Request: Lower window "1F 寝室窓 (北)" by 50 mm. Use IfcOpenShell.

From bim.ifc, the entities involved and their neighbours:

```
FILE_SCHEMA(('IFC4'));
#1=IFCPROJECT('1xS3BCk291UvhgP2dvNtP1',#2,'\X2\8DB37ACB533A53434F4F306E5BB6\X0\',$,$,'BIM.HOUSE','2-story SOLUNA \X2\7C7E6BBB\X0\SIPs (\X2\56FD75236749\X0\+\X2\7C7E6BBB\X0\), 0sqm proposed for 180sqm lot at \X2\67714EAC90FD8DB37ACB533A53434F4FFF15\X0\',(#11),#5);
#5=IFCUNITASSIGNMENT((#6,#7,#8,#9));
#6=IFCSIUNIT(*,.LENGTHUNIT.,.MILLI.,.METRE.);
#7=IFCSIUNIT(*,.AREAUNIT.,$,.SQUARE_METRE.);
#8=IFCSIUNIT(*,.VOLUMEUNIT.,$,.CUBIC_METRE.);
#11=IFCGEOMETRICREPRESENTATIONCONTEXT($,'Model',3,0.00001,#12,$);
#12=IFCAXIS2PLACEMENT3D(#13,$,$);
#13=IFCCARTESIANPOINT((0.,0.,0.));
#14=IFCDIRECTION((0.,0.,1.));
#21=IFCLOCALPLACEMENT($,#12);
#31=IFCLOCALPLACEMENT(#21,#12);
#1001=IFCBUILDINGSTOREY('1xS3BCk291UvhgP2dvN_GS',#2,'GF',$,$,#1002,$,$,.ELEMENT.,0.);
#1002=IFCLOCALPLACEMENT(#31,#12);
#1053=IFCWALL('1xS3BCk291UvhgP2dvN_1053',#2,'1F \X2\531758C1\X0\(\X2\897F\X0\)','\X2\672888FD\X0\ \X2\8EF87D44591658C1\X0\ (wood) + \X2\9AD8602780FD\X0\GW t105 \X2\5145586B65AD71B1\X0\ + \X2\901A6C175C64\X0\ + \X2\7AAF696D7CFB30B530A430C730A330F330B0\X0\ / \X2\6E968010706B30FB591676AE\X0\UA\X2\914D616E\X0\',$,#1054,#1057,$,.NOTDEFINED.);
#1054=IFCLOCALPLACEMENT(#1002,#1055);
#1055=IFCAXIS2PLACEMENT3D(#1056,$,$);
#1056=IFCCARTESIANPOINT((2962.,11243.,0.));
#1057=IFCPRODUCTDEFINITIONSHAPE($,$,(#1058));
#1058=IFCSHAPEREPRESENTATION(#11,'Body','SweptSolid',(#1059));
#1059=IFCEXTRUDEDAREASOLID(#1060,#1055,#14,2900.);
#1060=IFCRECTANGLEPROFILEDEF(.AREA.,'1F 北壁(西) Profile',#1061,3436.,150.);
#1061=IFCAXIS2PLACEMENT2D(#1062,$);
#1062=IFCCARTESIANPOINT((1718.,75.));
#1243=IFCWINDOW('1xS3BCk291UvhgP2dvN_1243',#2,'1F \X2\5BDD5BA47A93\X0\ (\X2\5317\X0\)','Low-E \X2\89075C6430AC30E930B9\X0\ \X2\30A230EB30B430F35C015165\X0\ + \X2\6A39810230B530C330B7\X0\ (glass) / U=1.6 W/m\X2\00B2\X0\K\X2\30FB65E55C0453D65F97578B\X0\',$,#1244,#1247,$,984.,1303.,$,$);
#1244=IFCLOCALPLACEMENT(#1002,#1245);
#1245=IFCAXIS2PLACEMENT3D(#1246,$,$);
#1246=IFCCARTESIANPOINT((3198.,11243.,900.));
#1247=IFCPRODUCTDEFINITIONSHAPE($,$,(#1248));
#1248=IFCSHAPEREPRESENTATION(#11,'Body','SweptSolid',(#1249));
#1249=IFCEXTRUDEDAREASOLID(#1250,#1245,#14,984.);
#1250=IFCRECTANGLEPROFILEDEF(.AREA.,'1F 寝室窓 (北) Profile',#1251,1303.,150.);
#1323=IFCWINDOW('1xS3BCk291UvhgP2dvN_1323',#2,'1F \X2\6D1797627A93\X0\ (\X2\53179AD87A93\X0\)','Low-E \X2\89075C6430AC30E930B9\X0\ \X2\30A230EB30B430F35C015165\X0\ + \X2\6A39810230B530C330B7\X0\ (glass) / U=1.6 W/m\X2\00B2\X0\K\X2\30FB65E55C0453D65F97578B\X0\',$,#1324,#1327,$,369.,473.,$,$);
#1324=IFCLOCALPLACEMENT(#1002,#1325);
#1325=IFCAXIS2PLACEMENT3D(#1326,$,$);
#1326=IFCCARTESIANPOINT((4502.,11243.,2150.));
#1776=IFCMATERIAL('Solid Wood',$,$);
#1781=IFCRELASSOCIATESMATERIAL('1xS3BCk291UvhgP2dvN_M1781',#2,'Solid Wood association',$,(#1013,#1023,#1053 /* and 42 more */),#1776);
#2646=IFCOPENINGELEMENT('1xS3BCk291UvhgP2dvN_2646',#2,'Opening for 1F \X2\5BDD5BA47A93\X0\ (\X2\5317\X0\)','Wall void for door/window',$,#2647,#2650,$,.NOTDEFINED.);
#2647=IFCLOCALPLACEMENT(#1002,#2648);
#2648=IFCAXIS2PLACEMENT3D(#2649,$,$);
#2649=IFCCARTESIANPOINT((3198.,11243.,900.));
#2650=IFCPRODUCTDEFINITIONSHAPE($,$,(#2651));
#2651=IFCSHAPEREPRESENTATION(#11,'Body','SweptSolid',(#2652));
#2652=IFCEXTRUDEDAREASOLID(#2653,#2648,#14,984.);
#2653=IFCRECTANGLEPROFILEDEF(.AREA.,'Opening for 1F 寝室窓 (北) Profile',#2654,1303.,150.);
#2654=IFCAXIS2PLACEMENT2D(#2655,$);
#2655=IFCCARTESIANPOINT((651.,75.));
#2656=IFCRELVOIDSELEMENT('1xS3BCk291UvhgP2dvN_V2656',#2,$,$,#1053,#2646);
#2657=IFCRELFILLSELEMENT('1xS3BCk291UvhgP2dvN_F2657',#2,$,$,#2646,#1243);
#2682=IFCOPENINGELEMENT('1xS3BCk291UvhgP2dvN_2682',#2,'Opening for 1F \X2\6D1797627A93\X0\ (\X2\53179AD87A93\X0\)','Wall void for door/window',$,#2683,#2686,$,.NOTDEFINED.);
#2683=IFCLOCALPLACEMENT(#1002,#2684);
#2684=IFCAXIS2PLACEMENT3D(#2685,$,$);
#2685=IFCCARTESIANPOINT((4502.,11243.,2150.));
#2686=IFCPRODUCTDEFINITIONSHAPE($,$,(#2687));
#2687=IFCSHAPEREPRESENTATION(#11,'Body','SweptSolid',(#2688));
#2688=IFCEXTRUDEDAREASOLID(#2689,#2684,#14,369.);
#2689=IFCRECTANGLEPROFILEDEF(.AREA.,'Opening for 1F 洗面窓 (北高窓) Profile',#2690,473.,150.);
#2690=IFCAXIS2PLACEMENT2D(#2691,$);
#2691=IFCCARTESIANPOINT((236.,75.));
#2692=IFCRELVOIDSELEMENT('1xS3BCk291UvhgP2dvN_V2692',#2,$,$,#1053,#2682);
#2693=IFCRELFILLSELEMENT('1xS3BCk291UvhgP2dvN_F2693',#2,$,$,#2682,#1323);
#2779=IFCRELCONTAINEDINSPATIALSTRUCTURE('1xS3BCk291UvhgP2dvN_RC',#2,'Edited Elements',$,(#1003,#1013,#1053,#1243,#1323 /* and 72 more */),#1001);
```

```python
import numpy as np
import ifcopenshell
import ifcopenshell.api.geometry
import ifcopenshell.util.placement
import ifcopenshell.util.unit

model = ifcopenshell.open("bim.ifc")
unit_scale = ifcopenshell.util.unit.calculate_unit_scale(model)

window = model.by_guid("1xS3BCk291UvhgP2dvN_1243")
opening = window.FillsVoids[0].RelatingOpeningElement
dz = -0.05 / unit_scale

shift = np.array([0.0, 0.0, dz])
# The window is not placed relative to its opening, so move both.
for product in (opening, window):
    matrix = ifcopenshell.util.placement.get_local_placement(product.ObjectPlacement)
    matrix[:3, 3] += shift
    ifcopenshell.api.geometry.edit_object_placement(model, product=product, matrix=matrix, is_si=False)

print(f"moved by {dz * unit_scale:+.3f} m")

model.write("bim_edited.ifc")
```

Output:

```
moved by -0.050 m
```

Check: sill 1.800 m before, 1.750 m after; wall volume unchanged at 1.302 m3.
